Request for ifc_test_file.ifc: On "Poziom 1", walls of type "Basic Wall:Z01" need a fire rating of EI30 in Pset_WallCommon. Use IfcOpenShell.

First a look at what the model holds.

```python
import ifcopenshell
import ifcopenshell.util.element

model = ifcopenshell.open("ifc_test_file.ifc")
print(model.schema)
storey = next(s for s in model.by_type("IfcBuildingStorey") if s.Name == "Poziom 1")
walls = [e for e in ifcopenshell.util.element.get_decomposition(storey) if e.is_a("IfcWall")]
seen = {}
for e in walls:
    element_type = ifcopenshell.util.element.get_type(e)
    key = (element_type.Name if element_type != e and element_type else None, ifcopenshell.util.element.get_pset(e, "Pset_WallCommon", "FireRating"))
    seen[key] = seen.get(key, 0) + 1
for (name, value), count in sorted(seen.items(), key=str):
    print(count, "x", name, "|", value)
```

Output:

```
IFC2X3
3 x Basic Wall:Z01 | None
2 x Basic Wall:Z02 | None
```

```python
import ifcopenshell
import ifcopenshell.api.pset
import ifcopenshell.util.element

model = ifcopenshell.open("ifc_test_file.ifc")

storey = next(s for s in model.by_type("IfcBuildingStorey") if s.Name == "Poziom 1")
walls = [e for e in ifcopenshell.util.element.get_decomposition(storey) if e.is_a("IfcWall")]

count = 0
for e in walls:
    element_type = ifcopenshell.util.element.get_type(e)
    if element_type in (None, e) or element_type.Name != "Basic Wall:Z01":
        continue
    # add_pset returns the element's existing set when there is one.
    pset = ifcopenshell.api.pset.add_pset(model, product=e, name="Pset_WallCommon")
    ifcopenshell.api.pset.edit_pset(model, pset=pset, properties={"FireRating": "EI30"})
    count += 1

print(count, "walls updated")

model.write("ifc_test_file_v2.ifc")
```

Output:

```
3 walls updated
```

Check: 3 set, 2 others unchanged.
